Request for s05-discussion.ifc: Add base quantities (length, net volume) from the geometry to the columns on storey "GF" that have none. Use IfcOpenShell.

First a look at what the model holds.

```python
import ifcopenshell
import ifcopenshell.util.element
import ifcopenshell.util.unit

model = ifcopenshell.open("s05-discussion.ifc")
print(model.schema)
for unit_type in ("LENGTHUNIT", "AREAUNIT", "VOLUMEUNIT"):
    print(unit_type, ifcopenshell.util.unit.calculate_unit_scale(model, unit_type))
storey = next(s for s in model.by_type("IfcBuildingStorey") if s.Name == "GF")
columns = [e for e in ifcopenshell.util.element.get_decomposition(storey) if e.is_a("IfcColumn")]
for e in sorted(columns, key=lambda e: e.id()):
    print(e.id(), e.is_a(), e.Name, list(ifcopenshell.util.element.get_psets(e, qtos_only=True)), sep=" | ")
```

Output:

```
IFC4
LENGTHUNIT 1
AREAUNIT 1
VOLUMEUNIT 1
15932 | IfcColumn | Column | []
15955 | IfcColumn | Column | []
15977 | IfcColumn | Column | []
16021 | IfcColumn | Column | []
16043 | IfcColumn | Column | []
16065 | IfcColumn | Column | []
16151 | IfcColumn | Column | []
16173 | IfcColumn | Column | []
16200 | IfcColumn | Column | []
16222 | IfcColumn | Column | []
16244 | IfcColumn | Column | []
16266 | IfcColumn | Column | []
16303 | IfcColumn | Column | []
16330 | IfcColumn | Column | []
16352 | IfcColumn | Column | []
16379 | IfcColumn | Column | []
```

```python
import ifcopenshell
import ifcopenshell.api.pset
import ifcopenshell.geom
import ifcopenshell.util.element
import ifcopenshell.util.shape
import ifcopenshell.util.unit

model = ifcopenshell.open("s05-discussion.ifc")
unit_scale = ifcopenshell.util.unit.calculate_unit_scale(model)
volume_scale = ifcopenshell.util.unit.calculate_unit_scale(model, "VOLUMEUNIT")
settings = ifcopenshell.geom.settings()

storey = next(s for s in model.by_type("IfcBuildingStorey") if s.Name == "GF")
columns = [e for e in ifcopenshell.util.element.get_decomposition(storey) if e.is_a("IfcColumn")]

for e in sorted(columns, key=lambda e: e.id()):
    if ifcopenshell.util.element.get_psets(e, qtos_only=True, should_inherit=False):
        continue
    # Geometry comes back in metres, in the element's own axes.
    shape = ifcopenshell.geom.create_shape(settings, e)
    values = {
        "Length": ifcopenshell.util.shape.get_z(shape.geometry) / unit_scale,
        "NetVolume": ifcopenshell.util.shape.get_volume(shape.geometry) / volume_scale,
    }
    qto = ifcopenshell.api.pset.add_qto(model, product=e, name="Qto_ColumnBaseQuantities")
    ifcopenshell.api.pset.edit_qto(model, qto=qto, properties=values)
    print(e.id(), {k: round(v, 3) for k, v in values.items()})

model.write("s05-discussion_v2.ifc")
```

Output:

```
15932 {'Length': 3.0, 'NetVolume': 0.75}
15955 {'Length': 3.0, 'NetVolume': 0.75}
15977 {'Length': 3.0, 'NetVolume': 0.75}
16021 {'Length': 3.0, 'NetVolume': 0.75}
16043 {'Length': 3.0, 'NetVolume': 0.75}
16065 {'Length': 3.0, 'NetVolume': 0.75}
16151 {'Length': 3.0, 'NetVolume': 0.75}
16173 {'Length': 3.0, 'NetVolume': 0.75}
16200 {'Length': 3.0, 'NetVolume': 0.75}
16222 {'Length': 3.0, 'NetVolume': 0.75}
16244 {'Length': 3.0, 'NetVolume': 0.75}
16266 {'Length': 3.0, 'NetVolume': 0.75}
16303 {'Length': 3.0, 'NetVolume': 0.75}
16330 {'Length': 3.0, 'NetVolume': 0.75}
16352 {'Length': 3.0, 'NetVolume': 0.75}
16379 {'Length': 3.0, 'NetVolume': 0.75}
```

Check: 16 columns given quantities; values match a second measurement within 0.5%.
